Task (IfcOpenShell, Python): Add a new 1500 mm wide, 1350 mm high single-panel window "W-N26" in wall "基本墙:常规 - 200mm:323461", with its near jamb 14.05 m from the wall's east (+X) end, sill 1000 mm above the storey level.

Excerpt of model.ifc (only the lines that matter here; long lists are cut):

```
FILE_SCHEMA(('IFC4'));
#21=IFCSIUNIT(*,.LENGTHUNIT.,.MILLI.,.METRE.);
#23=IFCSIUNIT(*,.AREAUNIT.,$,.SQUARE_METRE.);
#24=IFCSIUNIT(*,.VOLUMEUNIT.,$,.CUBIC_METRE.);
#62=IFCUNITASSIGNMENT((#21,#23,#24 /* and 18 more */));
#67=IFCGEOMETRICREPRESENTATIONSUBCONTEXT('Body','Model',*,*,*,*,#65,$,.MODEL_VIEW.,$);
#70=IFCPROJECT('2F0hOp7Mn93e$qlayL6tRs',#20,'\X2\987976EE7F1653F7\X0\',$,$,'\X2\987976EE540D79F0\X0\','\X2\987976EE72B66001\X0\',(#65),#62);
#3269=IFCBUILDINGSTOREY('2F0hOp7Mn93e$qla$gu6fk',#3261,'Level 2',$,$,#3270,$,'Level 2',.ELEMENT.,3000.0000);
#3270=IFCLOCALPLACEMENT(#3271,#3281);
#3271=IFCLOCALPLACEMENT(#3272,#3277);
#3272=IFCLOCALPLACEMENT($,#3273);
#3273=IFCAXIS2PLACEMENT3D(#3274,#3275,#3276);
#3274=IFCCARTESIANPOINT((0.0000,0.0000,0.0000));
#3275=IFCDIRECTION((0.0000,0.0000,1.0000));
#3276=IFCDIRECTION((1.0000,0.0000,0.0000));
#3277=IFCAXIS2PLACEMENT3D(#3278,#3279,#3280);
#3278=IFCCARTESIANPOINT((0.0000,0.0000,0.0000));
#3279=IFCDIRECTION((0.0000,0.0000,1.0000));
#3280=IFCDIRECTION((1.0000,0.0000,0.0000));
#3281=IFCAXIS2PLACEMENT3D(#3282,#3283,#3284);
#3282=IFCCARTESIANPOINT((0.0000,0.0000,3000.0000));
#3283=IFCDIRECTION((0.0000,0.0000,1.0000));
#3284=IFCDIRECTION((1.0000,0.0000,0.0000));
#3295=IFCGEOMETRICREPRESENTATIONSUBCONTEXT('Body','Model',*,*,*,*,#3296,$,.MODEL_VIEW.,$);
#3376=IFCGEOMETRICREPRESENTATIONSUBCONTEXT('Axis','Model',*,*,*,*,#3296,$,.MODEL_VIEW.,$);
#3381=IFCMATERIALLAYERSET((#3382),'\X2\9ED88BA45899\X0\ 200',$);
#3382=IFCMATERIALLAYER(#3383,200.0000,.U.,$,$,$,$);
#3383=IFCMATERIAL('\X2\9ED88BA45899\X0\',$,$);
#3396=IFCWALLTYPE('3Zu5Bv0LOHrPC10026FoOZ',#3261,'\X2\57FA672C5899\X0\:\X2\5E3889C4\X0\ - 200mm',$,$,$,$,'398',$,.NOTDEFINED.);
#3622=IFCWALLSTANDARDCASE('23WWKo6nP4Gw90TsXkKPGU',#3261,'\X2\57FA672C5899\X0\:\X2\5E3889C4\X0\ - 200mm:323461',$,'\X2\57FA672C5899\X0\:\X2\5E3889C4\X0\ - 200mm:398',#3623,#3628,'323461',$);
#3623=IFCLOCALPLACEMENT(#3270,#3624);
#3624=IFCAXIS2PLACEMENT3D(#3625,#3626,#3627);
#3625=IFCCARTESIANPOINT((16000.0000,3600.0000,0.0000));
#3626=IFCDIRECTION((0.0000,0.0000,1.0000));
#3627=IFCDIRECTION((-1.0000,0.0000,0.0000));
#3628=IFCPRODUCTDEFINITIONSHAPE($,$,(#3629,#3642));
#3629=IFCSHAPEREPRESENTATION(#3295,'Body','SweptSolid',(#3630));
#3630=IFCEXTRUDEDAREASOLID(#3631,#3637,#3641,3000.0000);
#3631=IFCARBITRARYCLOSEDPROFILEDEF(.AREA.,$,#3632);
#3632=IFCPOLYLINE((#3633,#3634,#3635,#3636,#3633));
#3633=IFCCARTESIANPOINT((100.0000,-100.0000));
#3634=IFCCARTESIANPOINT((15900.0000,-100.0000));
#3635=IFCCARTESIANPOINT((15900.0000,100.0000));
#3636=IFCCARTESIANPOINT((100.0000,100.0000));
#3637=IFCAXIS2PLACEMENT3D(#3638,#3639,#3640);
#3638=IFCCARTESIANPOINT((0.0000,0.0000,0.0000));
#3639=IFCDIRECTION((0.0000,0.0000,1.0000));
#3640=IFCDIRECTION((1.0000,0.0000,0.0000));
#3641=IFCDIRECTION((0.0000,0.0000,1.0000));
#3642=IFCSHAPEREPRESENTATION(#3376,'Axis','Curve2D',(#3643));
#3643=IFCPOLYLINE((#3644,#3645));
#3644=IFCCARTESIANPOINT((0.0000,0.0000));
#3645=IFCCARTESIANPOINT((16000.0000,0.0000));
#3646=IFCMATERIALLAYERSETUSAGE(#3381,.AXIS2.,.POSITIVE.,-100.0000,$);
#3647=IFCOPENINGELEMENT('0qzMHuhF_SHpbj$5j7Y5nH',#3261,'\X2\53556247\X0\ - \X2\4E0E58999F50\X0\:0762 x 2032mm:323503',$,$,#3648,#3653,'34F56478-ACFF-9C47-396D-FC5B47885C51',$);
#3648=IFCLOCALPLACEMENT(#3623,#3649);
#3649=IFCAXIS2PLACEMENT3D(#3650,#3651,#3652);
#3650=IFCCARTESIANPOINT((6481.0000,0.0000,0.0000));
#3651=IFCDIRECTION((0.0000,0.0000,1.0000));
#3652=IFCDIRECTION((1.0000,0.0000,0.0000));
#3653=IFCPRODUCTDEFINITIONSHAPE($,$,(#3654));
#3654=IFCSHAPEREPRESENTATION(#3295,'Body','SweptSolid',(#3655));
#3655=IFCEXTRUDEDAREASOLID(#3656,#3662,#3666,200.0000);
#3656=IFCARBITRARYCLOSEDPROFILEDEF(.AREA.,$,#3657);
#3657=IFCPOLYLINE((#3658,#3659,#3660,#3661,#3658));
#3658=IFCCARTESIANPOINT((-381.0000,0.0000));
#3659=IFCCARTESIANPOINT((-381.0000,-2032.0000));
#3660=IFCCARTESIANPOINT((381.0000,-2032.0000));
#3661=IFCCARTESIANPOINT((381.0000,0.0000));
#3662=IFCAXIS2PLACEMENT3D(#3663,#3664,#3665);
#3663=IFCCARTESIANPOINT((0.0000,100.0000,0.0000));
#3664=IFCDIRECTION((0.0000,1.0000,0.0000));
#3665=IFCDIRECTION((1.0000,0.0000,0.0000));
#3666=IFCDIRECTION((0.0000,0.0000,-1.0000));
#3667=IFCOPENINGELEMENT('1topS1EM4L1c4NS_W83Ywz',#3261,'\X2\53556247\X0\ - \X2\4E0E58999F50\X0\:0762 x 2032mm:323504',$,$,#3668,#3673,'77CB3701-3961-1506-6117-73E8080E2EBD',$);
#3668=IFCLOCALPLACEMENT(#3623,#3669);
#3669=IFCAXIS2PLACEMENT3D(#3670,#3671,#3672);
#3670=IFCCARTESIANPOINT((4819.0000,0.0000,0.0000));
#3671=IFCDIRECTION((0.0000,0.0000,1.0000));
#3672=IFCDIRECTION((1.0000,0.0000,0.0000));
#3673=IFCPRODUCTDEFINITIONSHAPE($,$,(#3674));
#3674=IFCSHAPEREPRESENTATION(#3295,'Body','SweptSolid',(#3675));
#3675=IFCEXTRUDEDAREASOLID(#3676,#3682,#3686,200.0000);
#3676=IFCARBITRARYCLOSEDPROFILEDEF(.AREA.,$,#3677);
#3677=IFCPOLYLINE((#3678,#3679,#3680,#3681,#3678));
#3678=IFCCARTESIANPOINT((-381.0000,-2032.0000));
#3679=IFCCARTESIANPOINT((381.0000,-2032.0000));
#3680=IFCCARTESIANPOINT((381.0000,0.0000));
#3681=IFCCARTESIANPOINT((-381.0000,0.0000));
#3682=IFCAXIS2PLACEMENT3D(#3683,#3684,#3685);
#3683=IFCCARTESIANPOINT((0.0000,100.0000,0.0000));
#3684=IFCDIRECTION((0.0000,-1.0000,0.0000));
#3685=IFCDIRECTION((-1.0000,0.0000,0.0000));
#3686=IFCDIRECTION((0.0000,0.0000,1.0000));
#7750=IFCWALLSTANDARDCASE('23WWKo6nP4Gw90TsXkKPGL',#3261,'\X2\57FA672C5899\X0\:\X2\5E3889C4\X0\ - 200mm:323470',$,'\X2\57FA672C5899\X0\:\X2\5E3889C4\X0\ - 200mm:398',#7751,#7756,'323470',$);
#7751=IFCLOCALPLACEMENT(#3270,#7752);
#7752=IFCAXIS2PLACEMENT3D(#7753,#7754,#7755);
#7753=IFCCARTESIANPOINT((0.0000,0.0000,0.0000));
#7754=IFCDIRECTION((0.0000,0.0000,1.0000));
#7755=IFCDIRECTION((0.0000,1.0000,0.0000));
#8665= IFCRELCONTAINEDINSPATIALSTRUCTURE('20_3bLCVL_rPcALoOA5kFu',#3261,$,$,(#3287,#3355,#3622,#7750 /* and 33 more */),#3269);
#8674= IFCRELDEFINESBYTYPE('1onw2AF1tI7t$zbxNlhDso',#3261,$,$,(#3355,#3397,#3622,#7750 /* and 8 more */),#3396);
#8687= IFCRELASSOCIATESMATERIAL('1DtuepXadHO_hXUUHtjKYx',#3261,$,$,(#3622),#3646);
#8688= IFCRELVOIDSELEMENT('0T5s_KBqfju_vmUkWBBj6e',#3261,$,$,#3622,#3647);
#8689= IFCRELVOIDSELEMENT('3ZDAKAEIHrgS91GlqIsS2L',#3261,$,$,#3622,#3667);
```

```python
import numpy as np
import ifcopenshell
import ifcopenshell.api.feature
import ifcopenshell.api.geometry
import ifcopenshell.api.root
import ifcopenshell.api.spatial
import ifcopenshell.geom
import ifcopenshell.util.element
import ifcopenshell.util.placement
import ifcopenshell.util.representation
import ifcopenshell.util.shape
import ifcopenshell.util.unit

model = ifcopenshell.open("model.ifc")
unit_scale = ifcopenshell.util.unit.calculate_unit_scale(model)
settings = ifcopenshell.geom.settings()


def volume(element):
    """Net volume in cubic metres, openings subtracted."""
    shape = ifcopenshell.geom.create_shape(settings, element)
    return ifcopenshell.util.shape.get_volume(shape.geometry)


wall = model.by_id(3622)
storey = ifcopenshell.util.element.get_container(wall, ifc_class="IfcBuildingStorey")
context = ifcopenshell.util.representation.get_context(model, "Model", "Body", "MODEL_VIEW")
before = volume(wall)

width, height, from_end, sill = 1.5, 1.35, 14.05, 1  # metres

# The wall runs along its own X axis, and the end named is its -X end.
wall_shape = ifcopenshell.geom.create_shape(settings, wall)
x, y, z = ifcopenshell.util.shape.get_vertices(wall_shape.geometry).T
start = x.min() + from_end
face, thickness = float(y.min()), float(y.max() - y.min())
wall_matrix = ifcopenshell.util.placement.get_local_placement(wall.ObjectPlacement)
level = ifcopenshell.util.placement.get_local_placement(storey.ObjectPlacement)[2, 3]


def in_wall(x, y):
    """Placement at x, y metres in the wall's axes, at sill height."""
    matrix = wall_matrix.copy()
    matrix[:, 3] = wall_matrix @ np.array([x / unit_scale, y / unit_scale, 0.0, 1.0])
    matrix[2, 3] = level + sill / unit_scale
    return matrix


# Opening: a box that overshoots both wall faces by 50 mm.
opening = ifcopenshell.api.root.create_entity(model, ifc_class="IfcOpeningElement", predefined_type="OPENING")
box = ifcopenshell.api.geometry.add_wall_representation(
    model, context=context, length=width, height=height, thickness=thickness + 0.1
)
ifcopenshell.api.geometry.assign_representation(model, product=opening, representation=box)
ifcopenshell.api.geometry.edit_object_placement(model, product=opening, matrix=in_wall(start, face - 0.05), is_si=False)
ifcopenshell.api.feature.add_feature(model, feature=opening, element=wall)

window = ifcopenshell.api.root.create_entity(model, ifc_class="IfcWindow", name="W-N26", predefined_type="WINDOW")
window.OverallWidth, window.OverallHeight = width / unit_scale, height / unit_scale
window.PartitioningType = "SINGLE_PANEL"
body = ifcopenshell.api.geometry.add_window_representation(
    model,
    context=context,
    overall_width=window.OverallWidth,
    overall_height=window.OverallHeight,
    partition_type="SINGLE_PANEL",
)
ifcopenshell.api.geometry.assign_representation(model, product=window, representation=body)
ifcopenshell.api.spatial.assign_container(model, products=[window], relating_structure=storey)
ifcopenshell.api.feature.add_filling(model, opening=opening, element=window)

# Centre the window in the wall's thickness.
ifcopenshell.api.geometry.edit_object_placement(model, product=window, matrix=in_wall(start, face), is_si=False)
window_shape = ifcopenshell.geom.create_shape(settings, window)
depth = ifcopenshell.util.shape.get_vertices(window_shape.geometry)[:, 1]
offset = face + thickness / 2 - (depth.min() + depth.max()) / 2
ifcopenshell.api.geometry.edit_object_placement(model, product=window, matrix=in_wall(start, offset), is_si=False)

after = volume(wall)

print(f"wall volume {before:.3f} -> {after:.3f} m3")

model.write("model_rev.ifc")
```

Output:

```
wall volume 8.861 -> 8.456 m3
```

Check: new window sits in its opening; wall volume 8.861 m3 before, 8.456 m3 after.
